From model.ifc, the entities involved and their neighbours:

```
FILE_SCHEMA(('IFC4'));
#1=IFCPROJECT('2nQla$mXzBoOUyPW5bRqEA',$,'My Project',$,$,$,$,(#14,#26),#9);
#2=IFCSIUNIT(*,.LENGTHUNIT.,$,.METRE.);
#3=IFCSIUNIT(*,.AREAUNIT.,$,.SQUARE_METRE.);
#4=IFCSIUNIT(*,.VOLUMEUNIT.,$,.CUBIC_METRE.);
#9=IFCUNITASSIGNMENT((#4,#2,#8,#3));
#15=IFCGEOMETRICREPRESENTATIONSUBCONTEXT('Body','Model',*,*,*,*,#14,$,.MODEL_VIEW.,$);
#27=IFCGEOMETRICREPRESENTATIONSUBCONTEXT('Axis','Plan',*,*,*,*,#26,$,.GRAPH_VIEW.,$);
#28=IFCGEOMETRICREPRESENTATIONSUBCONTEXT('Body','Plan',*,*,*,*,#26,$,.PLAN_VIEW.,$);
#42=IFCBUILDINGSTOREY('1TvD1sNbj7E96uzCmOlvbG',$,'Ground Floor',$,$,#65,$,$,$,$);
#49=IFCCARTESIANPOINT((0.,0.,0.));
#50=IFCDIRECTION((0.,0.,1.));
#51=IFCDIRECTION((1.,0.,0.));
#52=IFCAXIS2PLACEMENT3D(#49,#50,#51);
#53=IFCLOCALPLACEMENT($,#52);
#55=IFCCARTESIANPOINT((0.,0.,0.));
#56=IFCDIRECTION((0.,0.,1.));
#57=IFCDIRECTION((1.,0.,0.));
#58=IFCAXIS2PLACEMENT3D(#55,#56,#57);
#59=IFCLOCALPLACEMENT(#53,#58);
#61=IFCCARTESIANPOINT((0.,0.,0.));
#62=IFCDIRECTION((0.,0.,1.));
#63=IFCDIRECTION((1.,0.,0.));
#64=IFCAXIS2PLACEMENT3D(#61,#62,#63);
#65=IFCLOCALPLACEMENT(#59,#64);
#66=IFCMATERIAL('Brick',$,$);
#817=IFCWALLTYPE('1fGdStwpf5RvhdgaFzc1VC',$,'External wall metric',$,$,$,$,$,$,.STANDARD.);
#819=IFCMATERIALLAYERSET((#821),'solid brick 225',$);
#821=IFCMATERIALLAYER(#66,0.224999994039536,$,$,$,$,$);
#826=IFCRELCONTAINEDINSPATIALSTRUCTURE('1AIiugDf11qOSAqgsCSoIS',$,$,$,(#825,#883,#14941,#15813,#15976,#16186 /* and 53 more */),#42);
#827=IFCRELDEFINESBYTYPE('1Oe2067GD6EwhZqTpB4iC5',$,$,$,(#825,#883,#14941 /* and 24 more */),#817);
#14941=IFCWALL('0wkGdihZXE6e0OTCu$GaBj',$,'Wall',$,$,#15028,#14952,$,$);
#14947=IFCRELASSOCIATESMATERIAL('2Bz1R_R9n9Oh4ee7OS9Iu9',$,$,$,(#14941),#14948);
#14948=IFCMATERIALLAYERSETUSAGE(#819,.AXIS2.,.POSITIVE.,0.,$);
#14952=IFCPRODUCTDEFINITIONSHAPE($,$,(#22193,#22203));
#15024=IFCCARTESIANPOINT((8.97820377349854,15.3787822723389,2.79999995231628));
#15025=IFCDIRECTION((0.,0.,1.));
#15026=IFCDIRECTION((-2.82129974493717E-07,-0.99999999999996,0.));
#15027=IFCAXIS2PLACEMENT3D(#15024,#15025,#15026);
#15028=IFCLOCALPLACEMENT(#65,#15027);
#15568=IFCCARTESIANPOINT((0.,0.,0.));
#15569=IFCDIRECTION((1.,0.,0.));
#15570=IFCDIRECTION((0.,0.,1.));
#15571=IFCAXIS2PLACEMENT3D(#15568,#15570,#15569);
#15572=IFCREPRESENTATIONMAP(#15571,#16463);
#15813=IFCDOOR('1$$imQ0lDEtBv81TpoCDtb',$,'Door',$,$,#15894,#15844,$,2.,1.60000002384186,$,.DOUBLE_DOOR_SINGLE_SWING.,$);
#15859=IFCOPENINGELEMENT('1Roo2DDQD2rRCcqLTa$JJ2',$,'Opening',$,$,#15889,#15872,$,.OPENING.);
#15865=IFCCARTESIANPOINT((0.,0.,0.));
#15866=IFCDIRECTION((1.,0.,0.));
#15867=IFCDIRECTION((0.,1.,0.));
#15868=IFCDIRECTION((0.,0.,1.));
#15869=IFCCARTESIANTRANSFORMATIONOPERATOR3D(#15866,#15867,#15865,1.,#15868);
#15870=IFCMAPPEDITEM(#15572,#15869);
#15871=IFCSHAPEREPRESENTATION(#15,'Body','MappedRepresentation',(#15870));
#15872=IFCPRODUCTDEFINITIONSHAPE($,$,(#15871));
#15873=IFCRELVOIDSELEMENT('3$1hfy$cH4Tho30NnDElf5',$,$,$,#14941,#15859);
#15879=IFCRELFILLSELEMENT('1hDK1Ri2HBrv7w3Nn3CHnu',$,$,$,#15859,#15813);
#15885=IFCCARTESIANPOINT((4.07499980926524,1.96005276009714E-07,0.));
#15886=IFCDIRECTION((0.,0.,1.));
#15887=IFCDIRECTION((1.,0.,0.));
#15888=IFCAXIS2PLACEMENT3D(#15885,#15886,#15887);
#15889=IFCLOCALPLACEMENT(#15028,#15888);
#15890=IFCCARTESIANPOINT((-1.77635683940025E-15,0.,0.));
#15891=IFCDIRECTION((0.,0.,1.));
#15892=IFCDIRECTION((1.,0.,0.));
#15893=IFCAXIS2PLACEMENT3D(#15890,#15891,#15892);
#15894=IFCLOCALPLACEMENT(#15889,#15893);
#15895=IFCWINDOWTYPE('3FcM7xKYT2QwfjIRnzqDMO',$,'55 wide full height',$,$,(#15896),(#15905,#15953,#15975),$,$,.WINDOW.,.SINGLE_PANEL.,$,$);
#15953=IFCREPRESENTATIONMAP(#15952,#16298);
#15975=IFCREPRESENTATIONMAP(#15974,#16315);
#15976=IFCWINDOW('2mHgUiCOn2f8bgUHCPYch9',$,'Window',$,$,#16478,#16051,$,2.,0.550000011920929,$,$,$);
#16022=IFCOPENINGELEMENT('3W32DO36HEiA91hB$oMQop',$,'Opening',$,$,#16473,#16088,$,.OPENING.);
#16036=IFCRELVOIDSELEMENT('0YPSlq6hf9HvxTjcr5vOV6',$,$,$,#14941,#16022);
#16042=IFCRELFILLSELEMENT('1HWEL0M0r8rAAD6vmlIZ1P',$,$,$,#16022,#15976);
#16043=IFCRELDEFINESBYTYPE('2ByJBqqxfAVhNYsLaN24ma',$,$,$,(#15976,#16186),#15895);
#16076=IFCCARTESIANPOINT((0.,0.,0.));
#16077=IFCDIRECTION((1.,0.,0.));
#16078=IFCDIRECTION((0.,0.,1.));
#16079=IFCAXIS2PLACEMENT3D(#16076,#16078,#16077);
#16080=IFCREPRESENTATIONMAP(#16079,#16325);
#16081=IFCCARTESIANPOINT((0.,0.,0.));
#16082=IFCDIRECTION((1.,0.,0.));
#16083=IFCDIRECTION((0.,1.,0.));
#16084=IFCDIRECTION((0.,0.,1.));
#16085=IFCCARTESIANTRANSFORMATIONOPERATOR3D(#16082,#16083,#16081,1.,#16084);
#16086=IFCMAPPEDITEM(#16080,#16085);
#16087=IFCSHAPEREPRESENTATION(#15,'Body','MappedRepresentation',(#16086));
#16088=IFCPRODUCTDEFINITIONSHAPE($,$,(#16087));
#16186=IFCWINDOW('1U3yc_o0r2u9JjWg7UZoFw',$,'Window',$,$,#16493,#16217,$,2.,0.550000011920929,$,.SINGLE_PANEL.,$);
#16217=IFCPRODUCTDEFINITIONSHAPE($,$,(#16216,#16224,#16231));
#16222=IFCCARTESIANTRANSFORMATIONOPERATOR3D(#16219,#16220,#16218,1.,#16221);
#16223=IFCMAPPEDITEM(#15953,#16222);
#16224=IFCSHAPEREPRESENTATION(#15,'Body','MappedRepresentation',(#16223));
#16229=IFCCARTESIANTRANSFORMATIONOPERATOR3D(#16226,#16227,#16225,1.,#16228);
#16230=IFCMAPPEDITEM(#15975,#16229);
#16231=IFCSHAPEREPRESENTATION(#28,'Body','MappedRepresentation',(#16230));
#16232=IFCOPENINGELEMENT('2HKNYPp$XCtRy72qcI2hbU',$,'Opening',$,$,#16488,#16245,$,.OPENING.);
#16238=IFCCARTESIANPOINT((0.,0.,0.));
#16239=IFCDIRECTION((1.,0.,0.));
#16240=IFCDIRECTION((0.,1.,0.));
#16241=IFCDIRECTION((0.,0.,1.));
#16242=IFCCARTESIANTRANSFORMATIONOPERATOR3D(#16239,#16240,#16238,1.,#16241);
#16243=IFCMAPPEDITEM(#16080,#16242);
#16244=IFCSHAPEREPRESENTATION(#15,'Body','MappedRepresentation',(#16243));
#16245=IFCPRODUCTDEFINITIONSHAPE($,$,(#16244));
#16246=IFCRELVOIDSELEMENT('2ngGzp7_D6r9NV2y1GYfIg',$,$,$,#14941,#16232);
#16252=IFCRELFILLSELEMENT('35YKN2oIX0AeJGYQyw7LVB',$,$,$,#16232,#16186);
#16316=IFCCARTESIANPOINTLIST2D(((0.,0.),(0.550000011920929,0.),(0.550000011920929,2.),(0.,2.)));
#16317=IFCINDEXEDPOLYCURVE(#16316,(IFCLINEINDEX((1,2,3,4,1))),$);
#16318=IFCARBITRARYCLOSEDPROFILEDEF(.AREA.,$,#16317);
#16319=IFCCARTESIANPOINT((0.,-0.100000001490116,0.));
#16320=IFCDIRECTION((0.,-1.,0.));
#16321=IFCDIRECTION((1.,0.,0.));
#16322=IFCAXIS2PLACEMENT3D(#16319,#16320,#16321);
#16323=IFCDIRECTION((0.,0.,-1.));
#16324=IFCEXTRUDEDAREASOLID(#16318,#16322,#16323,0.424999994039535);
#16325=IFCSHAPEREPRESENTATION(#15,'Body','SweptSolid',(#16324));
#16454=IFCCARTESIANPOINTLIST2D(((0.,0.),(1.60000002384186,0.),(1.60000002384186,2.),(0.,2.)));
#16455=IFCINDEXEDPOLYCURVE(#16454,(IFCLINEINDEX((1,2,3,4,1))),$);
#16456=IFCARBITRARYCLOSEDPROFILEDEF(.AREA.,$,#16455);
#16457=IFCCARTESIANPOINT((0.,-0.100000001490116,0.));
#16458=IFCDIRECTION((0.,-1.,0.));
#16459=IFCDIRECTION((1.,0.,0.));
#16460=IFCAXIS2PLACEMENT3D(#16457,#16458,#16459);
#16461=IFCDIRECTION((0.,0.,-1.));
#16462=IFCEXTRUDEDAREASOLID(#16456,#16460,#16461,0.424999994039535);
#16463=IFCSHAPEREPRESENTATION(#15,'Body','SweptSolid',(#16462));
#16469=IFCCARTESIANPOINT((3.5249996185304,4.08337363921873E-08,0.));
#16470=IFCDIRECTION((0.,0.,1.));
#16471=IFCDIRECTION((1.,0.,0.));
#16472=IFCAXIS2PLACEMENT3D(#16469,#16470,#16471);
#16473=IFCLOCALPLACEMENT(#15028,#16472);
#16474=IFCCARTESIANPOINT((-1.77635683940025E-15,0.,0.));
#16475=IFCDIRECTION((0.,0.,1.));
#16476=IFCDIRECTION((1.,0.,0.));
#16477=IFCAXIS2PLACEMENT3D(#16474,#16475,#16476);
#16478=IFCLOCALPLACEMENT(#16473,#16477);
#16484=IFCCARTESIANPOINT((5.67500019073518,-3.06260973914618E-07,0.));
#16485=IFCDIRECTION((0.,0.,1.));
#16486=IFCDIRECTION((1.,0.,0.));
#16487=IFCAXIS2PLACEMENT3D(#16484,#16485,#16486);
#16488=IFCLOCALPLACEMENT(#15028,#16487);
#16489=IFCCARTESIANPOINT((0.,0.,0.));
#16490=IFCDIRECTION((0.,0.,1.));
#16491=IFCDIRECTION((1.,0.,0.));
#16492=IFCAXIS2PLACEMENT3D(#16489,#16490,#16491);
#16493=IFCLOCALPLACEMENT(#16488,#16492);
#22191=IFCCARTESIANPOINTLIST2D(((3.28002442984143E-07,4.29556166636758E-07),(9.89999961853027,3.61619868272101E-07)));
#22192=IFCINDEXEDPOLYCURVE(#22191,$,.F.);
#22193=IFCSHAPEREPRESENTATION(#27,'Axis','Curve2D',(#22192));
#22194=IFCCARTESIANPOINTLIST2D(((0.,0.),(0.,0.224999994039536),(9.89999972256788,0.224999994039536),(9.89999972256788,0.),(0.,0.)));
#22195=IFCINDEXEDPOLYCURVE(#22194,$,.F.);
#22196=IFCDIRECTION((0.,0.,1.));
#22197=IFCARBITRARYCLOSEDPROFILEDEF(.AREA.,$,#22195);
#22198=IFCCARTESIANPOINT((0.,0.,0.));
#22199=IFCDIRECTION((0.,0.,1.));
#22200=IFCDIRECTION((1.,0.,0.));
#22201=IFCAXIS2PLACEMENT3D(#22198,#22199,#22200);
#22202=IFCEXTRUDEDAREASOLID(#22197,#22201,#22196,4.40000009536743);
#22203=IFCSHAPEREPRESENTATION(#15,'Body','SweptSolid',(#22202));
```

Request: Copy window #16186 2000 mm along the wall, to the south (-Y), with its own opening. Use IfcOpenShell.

```python
import ifcopenshell
import ifcopenshell.api.feature
import ifcopenshell.api.geometry
import ifcopenshell.api.root
import ifcopenshell.geom
import ifcopenshell.util.element
import ifcopenshell.util.placement
import ifcopenshell.util.shape
import ifcopenshell.util.unit

model = ifcopenshell.open("model.ifc")
unit_scale = ifcopenshell.util.unit.calculate_unit_scale(model)
settings = ifcopenshell.geom.settings()


def volume(element):
    """Net volume in cubic metres, openings subtracted."""
    shape = ifcopenshell.geom.create_shape(settings, element)
    return ifcopenshell.util.shape.get_volume(shape.geometry)


window = model.by_guid("1U3yc_o0r2u9JjWg7UZoFw")
opening = window.FillsVoids[0].RelatingOpeningElement
wall = opening.VoidsElements[0].RelatingBuildingElement
before = volume(wall)
shift = ifcopenshell.util.placement.get_local_placement(wall.ObjectPlacement)[:3, 0] * 2 / unit_scale

# copy_class copies the void relationship, type, container and properties, but no geometry.
new_opening = ifcopenshell.api.root.copy_class(model, product=opening)
new_opening.Representation = ifcopenshell.util.element.copy_deep(
    model, opening.Representation, exclude=["IfcGeometricRepresentationContext", "IfcRepresentationMap"]
)
new_window = ifcopenshell.api.root.copy_class(model, product=window)
new_window.Representation = ifcopenshell.util.element.copy_deep(
    model, window.Representation, exclude=["IfcGeometricRepresentationContext", "IfcRepresentationMap"]
)
ifcopenshell.api.feature.add_filling(model, opening=new_opening, element=new_window)

for old, new in ((opening, new_opening), (window, new_window)):
    matrix = ifcopenshell.util.placement.get_local_placement(old.ObjectPlacement)
    matrix[:3, 3] += shift
    ifcopenshell.api.geometry.edit_object_placement(model, product=new, matrix=matrix, is_si=False)

after = volume(wall)

print(f"wall volume {before:.3f} -> {after:.3f} m3")

model.write("model-out.ifc")
```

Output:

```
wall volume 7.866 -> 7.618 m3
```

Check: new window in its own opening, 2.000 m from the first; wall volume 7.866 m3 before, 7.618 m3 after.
